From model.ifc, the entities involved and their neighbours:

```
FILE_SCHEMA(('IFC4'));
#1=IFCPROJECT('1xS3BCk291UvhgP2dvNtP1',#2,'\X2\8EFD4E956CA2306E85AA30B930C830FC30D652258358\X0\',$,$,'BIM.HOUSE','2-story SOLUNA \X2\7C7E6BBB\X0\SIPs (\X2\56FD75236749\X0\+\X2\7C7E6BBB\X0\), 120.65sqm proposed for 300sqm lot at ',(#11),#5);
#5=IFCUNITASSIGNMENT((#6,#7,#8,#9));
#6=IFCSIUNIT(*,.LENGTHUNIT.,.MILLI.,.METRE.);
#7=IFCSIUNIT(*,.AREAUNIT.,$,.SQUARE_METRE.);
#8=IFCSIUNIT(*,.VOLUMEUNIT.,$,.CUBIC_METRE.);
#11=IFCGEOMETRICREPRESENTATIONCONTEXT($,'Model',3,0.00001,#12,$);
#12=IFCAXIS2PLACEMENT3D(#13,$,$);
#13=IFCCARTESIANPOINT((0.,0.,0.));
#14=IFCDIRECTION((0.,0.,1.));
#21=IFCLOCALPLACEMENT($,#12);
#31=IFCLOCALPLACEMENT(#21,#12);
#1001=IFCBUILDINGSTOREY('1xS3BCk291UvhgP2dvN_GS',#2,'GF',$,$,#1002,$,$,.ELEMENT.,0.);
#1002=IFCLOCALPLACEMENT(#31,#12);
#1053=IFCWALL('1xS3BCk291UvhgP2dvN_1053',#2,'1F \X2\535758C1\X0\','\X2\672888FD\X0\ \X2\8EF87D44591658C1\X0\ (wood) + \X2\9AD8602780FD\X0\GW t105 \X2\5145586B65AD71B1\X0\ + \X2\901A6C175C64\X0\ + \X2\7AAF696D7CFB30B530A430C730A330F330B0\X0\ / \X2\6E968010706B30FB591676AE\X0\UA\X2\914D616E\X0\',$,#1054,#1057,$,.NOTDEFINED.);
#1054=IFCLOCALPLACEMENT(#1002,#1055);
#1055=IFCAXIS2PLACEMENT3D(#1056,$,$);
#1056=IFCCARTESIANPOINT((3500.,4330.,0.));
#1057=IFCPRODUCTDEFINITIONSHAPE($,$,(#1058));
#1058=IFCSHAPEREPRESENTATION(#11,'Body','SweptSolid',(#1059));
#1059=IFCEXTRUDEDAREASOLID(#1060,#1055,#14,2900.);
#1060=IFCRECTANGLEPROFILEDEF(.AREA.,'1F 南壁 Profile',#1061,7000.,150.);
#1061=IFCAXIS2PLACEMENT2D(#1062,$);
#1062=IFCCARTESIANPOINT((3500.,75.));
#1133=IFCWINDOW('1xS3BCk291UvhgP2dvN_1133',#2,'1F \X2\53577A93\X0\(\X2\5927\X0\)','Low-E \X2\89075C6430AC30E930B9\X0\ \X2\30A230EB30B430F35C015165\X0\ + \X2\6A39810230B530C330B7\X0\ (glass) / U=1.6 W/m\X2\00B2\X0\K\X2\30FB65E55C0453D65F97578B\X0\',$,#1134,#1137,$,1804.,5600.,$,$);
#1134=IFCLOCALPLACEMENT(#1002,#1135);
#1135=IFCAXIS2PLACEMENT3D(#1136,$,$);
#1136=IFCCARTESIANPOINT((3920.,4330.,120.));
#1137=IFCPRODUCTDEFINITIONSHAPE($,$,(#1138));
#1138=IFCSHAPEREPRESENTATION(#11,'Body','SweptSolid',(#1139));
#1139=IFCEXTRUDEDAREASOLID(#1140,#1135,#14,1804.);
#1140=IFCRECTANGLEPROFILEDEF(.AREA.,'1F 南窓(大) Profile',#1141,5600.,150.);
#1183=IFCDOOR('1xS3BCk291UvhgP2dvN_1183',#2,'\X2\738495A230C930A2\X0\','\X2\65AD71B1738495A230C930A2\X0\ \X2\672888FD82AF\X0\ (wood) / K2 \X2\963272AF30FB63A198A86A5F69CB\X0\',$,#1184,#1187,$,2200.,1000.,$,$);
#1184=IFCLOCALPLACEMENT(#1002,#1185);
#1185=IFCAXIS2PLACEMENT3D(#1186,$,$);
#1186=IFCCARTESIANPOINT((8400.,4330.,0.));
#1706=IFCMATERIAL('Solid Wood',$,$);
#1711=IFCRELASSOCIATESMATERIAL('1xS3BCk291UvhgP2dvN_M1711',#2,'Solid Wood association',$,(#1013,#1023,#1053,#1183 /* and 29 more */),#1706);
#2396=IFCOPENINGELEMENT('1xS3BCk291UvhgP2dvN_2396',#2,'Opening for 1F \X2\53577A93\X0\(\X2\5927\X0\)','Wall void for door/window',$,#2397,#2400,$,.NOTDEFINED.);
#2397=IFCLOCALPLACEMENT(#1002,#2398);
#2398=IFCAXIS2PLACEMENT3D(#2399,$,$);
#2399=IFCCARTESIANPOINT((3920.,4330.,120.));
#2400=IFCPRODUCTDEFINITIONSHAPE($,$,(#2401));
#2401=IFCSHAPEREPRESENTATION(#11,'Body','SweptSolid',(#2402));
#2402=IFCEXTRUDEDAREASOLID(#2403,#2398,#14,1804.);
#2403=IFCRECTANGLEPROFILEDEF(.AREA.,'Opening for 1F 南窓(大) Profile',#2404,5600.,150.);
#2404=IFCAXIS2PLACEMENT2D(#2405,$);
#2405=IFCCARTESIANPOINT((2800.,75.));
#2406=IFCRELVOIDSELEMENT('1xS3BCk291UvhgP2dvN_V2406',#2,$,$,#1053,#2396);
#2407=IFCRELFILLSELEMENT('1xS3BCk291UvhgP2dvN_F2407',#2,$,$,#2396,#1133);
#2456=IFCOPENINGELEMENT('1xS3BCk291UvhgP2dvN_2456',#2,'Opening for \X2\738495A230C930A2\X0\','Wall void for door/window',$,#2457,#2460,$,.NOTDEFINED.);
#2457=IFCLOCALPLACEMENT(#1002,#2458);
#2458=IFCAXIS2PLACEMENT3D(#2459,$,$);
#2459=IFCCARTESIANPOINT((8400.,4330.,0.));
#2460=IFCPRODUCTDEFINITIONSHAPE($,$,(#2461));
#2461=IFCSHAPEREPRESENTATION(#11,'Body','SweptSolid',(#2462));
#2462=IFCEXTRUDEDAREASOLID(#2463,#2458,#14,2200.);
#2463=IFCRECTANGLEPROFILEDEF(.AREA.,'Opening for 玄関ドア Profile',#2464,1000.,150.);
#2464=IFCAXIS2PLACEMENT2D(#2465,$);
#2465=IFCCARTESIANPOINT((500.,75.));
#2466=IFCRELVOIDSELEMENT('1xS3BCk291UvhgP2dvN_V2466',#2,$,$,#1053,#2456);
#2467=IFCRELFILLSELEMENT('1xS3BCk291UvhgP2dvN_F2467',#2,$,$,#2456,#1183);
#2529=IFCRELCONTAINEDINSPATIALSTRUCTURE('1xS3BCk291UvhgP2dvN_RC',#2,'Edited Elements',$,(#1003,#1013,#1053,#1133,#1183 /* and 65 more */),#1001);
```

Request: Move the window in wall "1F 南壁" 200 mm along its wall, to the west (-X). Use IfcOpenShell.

```python
import ifcopenshell
import ifcopenshell.api.geometry
import ifcopenshell.util.placement
import ifcopenshell.util.unit

model = ifcopenshell.open("model.ifc")
unit_scale = ifcopenshell.util.unit.calculate_unit_scale(model)

window = model.by_guid("1xS3BCk291UvhgP2dvN_1133")
opening = window.FillsVoids[0].RelatingOpeningElement
wall = opening.VoidsElements[0].RelatingBuildingElement

wall_matrix = ifcopenshell.util.placement.get_local_placement(wall.ObjectPlacement)
shift = wall_matrix[:3, 0] * -0.2 / unit_scale
before = ifcopenshell.util.placement.get_local_placement(window.ObjectPlacement)[:3, 3].copy()

# The window is not placed relative to its opening, so move both.
for product in (opening, window):
    matrix = ifcopenshell.util.placement.get_local_placement(product.ObjectPlacement)
    matrix[:3, 3] += shift
    ifcopenshell.api.geometry.edit_object_placement(model, product=product, matrix=matrix, is_si=False)

after = ifcopenshell.util.placement.get_local_placement(window.ObjectPlacement)[:3, 3]
print("window moved by", (after - before).round(3) + 0.0)

model.write("model_edited.ifc")
```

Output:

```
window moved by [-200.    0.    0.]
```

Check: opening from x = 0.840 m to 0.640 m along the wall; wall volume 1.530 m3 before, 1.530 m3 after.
